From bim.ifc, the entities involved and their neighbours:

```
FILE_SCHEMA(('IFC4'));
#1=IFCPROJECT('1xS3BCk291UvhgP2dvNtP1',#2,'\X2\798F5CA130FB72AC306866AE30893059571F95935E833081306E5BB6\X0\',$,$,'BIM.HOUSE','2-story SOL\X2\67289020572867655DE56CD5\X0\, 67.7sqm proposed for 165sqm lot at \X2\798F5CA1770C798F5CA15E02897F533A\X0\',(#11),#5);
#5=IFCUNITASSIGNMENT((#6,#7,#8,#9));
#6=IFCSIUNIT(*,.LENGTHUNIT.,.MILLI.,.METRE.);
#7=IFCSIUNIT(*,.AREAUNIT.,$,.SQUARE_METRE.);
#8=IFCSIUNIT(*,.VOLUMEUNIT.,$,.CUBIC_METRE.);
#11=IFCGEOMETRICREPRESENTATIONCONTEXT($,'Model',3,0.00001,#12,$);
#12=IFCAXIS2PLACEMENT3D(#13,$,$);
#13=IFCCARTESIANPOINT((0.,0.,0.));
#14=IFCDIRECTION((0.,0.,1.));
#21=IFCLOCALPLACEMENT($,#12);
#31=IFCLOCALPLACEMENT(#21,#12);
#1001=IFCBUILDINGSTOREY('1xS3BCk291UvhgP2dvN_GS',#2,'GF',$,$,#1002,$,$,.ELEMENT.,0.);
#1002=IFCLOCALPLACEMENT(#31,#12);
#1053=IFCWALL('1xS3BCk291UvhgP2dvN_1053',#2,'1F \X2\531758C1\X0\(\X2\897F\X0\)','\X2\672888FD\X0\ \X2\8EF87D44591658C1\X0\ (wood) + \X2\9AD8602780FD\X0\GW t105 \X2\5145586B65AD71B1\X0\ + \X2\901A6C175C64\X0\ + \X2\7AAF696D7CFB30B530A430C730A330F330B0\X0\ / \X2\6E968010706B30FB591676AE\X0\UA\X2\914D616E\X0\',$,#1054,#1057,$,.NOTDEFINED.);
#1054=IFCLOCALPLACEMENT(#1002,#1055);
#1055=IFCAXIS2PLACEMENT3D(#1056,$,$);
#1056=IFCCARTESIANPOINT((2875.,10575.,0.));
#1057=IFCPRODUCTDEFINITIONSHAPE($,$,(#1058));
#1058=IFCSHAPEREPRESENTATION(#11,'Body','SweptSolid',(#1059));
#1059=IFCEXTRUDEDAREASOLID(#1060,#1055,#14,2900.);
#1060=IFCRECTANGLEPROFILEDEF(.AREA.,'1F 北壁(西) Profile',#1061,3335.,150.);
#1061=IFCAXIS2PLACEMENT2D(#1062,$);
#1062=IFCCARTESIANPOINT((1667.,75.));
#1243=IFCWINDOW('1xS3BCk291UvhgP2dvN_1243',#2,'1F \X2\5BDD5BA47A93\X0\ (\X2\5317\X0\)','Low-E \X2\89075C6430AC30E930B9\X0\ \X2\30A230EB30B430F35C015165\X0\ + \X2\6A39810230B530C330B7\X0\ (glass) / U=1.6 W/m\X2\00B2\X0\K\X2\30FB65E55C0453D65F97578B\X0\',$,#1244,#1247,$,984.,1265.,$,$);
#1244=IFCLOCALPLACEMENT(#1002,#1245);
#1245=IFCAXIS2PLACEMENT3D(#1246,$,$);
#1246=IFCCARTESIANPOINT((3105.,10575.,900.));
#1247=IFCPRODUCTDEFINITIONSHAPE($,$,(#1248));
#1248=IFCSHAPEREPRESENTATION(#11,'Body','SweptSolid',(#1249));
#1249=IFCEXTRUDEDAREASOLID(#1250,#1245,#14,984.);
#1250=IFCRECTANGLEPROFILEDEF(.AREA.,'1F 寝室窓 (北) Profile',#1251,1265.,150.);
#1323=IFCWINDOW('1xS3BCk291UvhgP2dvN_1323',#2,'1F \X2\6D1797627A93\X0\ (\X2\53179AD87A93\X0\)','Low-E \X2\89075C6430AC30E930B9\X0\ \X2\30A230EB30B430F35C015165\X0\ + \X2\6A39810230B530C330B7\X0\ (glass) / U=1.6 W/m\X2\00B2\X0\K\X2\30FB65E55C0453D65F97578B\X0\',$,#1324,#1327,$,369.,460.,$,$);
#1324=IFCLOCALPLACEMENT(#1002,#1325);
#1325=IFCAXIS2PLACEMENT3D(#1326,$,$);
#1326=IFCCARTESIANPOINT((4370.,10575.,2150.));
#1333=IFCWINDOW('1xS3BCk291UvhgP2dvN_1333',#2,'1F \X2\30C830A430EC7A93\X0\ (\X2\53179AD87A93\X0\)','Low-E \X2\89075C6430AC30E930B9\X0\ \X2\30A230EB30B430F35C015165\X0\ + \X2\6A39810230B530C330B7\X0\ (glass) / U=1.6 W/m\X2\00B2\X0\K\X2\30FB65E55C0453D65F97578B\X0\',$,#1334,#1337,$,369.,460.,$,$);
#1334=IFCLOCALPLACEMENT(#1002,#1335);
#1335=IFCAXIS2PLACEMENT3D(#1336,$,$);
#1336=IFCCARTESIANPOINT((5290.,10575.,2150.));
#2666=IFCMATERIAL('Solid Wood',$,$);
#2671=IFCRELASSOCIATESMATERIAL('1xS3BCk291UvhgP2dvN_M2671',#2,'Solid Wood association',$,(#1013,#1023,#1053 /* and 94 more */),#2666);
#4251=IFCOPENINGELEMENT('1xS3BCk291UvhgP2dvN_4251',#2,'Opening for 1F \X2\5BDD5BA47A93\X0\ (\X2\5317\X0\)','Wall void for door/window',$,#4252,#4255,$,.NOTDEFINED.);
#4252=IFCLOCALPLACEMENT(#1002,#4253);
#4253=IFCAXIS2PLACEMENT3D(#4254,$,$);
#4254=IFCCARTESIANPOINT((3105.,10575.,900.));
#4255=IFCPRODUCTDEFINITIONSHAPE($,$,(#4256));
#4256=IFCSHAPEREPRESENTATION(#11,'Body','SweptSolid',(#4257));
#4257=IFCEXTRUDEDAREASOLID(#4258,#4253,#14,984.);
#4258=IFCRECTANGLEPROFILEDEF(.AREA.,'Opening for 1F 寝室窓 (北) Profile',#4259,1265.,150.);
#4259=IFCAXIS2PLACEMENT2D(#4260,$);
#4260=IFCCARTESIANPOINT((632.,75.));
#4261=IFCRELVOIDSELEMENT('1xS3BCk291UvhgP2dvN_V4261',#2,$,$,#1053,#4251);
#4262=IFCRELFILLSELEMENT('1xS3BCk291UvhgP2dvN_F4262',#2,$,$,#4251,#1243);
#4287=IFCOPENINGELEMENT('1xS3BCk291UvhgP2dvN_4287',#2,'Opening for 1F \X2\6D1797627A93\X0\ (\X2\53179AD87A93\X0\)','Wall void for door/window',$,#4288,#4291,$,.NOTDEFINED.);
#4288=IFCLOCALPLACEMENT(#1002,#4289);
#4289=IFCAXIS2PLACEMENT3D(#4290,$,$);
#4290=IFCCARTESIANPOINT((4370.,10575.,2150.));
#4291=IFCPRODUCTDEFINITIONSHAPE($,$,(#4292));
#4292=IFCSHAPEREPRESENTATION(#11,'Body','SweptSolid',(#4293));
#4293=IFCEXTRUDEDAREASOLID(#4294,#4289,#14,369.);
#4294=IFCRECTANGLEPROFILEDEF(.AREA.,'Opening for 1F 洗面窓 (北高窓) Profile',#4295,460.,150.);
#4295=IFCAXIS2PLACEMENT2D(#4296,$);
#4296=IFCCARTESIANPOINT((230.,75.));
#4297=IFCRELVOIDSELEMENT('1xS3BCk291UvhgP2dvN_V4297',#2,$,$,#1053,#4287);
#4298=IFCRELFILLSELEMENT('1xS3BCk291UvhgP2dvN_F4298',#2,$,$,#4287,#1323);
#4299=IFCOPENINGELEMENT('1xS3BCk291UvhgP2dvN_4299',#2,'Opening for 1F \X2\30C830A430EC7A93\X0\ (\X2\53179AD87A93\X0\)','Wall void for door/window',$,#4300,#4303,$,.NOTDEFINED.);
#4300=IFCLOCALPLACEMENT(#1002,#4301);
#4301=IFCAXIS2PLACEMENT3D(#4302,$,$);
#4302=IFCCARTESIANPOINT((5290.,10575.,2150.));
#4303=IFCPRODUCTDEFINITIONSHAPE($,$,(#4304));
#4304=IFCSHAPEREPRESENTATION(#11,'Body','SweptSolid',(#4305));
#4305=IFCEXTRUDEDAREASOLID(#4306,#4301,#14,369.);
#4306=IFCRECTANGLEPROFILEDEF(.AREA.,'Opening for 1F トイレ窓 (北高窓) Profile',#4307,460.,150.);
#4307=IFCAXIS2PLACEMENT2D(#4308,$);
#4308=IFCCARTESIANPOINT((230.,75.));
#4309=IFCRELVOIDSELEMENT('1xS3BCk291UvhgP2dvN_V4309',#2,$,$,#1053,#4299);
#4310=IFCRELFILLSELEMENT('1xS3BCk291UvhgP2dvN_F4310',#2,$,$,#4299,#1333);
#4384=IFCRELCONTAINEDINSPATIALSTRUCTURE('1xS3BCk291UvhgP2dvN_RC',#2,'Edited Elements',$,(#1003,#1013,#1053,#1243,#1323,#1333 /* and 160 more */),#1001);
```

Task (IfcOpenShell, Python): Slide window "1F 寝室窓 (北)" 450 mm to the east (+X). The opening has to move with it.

```python
import ifcopenshell
import ifcopenshell.api.geometry
import ifcopenshell.util.placement
import ifcopenshell.util.unit

model = ifcopenshell.open("bim.ifc")
unit_scale = ifcopenshell.util.unit.calculate_unit_scale(model)

window = model.by_id(1243)
opening = window.FillsVoids[0].RelatingOpeningElement
wall = opening.VoidsElements[0].RelatingBuildingElement

wall_matrix = ifcopenshell.util.placement.get_local_placement(wall.ObjectPlacement)
shift = wall_matrix[:3, 0] * 0.45 / unit_scale
before = ifcopenshell.util.placement.get_local_placement(window.ObjectPlacement)[:3, 3].copy()

# The window is not placed relative to its opening, so move both.
for product in (opening, window):
    matrix = ifcopenshell.util.placement.get_local_placement(product.ObjectPlacement)
    matrix[:3, 3] += shift
    ifcopenshell.api.geometry.edit_object_placement(model, product=product, matrix=matrix, is_si=False)

after = ifcopenshell.util.placement.get_local_placement(window.ObjectPlacement)[:3, 3]
print("window moved by", (after - before).round(3) + 0.0)

model.write("bim_edited.ifc")
```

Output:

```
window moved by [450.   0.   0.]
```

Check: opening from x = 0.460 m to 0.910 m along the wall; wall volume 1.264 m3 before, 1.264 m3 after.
